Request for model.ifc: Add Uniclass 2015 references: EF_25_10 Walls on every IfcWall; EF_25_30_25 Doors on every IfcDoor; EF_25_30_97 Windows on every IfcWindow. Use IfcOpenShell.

First a look at what the model holds.

```python
import ifcopenshell

model = ifcopenshell.open("model.ifc")
print(model.schema)
print("classifications:", [c.Name for c in model.by_type("IfcClassification")])
for ifc_class in ("IfcDoor", "IfcRoof", "IfcStair", "IfcWall", "IfcWindow"):
    print(ifc_class, len(model.by_type(ifc_class)))
```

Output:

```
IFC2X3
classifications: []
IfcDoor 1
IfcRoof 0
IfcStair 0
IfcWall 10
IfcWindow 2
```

```python
import ifcopenshell
import ifcopenshell.api.classification

model = ifcopenshell.open("model.ifc")

# IFC2X3 requires Source and Edition and has no link from the project to the system.
system = model.create_entity("IfcClassification", Source="NBS", Edition="2015", Name="Uniclass 2015")

codes = {
    "IfcWall": ("EF_25_10", "Walls"),
    "IfcDoor": ("EF_25_30_25", "Doors"),
    "IfcWindow": ("EF_25_30_97", "Windows"),
}
for ifc_class, (code, name) in codes.items():
    products = model.by_type(ifc_class)
    ifcopenshell.api.classification.add_reference(
        model, products=products, classification=system, identification=code, name=name
    )
    print(code, len(products))

model.write("model_edited.ifc")
```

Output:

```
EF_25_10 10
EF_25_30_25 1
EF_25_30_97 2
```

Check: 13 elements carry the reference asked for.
